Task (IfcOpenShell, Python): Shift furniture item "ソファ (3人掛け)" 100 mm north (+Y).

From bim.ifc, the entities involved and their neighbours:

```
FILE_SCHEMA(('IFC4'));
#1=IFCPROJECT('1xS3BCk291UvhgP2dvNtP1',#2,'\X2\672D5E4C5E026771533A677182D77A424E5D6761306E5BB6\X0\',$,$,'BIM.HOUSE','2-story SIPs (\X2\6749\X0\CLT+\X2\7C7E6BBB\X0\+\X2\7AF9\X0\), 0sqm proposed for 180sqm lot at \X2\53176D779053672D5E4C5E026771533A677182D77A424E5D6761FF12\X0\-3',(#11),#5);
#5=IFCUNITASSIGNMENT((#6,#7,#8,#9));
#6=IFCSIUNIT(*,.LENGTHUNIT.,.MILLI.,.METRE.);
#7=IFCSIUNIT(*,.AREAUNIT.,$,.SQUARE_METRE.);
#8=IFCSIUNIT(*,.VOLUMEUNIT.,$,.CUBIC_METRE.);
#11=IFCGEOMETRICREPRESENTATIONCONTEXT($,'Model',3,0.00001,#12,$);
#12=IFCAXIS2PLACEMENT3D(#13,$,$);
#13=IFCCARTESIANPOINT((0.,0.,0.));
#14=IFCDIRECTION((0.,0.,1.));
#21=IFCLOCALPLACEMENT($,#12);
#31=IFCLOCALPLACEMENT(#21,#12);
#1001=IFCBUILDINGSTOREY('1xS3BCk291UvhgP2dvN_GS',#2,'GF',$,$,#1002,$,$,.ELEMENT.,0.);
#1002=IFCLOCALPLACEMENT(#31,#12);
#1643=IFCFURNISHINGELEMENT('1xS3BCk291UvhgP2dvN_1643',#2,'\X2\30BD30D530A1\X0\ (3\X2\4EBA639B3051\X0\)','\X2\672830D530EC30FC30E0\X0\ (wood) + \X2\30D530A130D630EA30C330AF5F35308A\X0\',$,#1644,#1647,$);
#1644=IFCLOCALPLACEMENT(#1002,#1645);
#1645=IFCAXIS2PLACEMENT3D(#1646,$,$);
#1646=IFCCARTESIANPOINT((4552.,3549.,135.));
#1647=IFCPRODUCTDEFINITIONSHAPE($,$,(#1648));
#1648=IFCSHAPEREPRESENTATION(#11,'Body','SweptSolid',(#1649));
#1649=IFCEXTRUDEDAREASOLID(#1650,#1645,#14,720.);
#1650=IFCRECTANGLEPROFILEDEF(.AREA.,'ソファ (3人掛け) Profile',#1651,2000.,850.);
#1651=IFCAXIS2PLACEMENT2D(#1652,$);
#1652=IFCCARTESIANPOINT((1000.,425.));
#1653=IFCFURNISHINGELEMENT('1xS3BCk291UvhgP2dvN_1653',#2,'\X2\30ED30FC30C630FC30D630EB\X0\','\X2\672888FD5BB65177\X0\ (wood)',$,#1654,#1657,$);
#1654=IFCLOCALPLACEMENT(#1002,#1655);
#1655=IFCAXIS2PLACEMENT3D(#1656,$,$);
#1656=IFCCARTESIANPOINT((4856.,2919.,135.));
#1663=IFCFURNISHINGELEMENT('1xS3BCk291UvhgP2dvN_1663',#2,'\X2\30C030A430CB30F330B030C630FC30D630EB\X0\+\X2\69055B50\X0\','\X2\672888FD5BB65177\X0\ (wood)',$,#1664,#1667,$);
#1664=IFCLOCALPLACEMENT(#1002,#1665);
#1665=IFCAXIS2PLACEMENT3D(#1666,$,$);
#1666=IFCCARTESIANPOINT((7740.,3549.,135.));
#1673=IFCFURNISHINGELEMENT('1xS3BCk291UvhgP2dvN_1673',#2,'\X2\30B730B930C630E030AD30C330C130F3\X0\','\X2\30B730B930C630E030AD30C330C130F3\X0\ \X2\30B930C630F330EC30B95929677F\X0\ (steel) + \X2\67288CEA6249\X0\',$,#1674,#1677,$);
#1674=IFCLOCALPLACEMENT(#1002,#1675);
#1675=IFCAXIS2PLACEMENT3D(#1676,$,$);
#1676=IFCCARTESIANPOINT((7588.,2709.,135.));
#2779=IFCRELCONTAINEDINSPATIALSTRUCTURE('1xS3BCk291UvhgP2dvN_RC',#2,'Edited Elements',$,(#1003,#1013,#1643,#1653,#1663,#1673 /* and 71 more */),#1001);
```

```python
import ifcopenshell
import ifcopenshell.api.geometry
import ifcopenshell.util.placement

model = ifcopenshell.open("bim.ifc")

item = model.by_guid("1xS3BCk291UvhgP2dvN_1643")
matrix = ifcopenshell.util.placement.get_local_placement(item.ObjectPlacement)
matrix[1, 3] += 100.0
ifcopenshell.api.geometry.edit_object_placement(model, product=item, matrix=matrix, is_si=False)

print(ifcopenshell.util.placement.get_local_placement(item.ObjectPlacement).round(3) + 0.0)

model.write("bim_edited.ifc")
```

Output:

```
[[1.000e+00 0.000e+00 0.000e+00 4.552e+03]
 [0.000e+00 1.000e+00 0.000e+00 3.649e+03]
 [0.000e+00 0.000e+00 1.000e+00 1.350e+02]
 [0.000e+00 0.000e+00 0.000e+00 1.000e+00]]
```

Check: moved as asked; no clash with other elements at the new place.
